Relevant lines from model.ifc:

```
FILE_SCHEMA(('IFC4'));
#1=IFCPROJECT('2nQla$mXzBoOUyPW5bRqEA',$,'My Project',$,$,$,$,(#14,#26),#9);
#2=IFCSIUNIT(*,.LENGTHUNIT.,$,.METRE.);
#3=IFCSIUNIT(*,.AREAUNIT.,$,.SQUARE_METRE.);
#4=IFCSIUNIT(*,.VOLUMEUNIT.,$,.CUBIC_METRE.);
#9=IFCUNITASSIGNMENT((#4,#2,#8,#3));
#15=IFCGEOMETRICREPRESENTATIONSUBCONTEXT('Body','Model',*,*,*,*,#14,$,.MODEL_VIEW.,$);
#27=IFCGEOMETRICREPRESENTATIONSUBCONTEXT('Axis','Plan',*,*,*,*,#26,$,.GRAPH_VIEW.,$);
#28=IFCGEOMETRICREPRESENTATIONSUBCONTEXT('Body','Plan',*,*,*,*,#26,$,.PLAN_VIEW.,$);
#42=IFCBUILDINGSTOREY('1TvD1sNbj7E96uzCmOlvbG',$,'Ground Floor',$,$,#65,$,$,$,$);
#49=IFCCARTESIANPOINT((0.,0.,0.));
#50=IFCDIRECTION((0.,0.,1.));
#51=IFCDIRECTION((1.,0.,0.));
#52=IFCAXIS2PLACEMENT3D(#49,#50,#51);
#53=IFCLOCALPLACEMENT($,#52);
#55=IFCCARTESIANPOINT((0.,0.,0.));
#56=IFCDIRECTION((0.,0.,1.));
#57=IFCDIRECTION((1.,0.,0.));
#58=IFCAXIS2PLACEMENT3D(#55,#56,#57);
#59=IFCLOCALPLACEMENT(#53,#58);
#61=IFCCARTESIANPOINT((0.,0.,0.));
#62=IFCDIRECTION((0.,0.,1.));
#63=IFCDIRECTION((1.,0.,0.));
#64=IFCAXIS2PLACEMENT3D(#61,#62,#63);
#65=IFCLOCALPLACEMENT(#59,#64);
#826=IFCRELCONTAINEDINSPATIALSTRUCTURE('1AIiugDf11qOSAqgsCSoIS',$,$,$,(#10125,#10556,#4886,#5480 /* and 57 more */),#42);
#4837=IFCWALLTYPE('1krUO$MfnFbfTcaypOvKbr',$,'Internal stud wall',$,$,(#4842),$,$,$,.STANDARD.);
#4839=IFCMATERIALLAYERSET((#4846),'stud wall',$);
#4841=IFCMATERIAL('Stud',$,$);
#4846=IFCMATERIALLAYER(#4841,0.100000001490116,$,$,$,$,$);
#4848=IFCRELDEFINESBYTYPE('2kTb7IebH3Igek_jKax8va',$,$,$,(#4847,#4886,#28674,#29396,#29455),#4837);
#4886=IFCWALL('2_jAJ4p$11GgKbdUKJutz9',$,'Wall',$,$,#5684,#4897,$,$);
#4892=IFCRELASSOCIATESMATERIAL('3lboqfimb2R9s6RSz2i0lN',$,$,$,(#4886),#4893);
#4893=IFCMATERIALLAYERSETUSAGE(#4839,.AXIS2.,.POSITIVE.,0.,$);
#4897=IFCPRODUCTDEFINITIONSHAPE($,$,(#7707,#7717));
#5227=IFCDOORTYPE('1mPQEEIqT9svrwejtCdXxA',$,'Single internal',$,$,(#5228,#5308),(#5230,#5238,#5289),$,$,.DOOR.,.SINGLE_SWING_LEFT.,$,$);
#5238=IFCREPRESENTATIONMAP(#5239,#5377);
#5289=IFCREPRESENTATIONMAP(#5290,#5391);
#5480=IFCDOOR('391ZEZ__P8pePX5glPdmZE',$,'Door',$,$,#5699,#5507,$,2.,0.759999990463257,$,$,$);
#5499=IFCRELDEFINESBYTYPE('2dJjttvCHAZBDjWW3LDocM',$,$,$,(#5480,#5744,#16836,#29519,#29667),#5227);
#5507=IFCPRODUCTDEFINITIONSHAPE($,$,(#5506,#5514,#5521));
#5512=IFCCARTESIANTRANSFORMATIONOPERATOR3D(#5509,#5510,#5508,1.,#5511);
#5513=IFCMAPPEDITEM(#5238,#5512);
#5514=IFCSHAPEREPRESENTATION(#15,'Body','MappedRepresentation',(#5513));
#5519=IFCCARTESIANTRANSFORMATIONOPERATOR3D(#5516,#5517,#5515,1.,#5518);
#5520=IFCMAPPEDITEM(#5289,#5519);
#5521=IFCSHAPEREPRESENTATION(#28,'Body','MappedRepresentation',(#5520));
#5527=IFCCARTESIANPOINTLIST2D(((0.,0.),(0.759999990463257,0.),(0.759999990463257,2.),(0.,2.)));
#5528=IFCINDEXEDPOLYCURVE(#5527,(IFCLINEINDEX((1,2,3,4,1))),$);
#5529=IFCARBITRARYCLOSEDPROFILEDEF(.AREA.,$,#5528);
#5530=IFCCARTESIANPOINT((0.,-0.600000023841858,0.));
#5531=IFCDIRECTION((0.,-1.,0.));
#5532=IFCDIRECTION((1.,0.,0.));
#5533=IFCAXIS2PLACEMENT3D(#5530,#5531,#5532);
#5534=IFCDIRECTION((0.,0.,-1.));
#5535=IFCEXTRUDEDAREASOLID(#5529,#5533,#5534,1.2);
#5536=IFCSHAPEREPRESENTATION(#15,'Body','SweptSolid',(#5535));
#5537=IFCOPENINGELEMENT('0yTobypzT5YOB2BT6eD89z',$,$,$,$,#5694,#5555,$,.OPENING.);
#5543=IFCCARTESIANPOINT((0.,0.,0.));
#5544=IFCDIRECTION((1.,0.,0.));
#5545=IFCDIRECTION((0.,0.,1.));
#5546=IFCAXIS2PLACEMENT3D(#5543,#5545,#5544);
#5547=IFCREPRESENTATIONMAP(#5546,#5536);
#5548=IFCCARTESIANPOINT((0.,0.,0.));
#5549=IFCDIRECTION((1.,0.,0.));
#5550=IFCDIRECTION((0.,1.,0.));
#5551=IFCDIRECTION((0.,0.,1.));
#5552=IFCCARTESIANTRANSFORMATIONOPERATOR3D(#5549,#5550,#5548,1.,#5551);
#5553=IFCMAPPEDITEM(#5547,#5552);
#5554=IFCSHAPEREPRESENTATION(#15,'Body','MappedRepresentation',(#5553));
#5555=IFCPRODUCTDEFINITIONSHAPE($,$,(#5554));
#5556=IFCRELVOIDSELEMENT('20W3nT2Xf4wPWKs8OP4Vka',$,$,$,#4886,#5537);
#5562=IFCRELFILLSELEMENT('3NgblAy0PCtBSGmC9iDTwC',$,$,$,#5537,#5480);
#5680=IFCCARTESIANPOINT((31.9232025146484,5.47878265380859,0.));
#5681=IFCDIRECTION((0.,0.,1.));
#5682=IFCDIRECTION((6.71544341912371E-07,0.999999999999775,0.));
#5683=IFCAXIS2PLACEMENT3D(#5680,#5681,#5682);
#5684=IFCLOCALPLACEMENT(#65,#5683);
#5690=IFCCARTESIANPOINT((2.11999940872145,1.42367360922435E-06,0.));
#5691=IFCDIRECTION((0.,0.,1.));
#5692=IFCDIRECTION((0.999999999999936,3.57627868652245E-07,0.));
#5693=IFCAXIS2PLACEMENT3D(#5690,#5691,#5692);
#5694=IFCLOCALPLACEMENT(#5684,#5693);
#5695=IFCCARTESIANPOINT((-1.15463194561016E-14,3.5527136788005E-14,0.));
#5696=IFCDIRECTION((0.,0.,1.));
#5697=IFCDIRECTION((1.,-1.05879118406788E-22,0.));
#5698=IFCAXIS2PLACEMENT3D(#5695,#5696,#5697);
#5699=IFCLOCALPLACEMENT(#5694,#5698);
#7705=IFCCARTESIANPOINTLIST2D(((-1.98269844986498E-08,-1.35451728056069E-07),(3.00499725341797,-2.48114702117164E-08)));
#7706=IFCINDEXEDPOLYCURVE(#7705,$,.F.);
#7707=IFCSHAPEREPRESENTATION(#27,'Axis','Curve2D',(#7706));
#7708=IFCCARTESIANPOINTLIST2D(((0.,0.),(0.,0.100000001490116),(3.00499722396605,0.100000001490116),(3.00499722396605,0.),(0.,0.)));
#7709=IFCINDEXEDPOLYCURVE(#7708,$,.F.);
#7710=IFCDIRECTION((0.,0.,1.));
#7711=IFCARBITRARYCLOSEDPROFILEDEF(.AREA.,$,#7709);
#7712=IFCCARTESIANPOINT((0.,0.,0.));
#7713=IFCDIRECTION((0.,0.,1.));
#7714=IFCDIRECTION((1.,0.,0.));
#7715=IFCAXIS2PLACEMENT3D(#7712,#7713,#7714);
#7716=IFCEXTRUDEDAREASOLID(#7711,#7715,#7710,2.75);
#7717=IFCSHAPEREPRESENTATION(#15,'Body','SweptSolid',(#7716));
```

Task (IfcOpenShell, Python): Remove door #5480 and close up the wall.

```python
import ifcopenshell
import ifcopenshell.api.feature
import ifcopenshell.api.root
import ifcopenshell.geom
import ifcopenshell.util.shape

model = ifcopenshell.open("model.ifc")
settings = ifcopenshell.geom.settings()


def volume(element):
    """Net volume in cubic metres, openings subtracted."""
    shape = ifcopenshell.geom.create_shape(settings, element)
    return ifcopenshell.util.shape.get_volume(shape.geometry)


door = model.by_guid("391ZEZ__P8pePX5glPdmZE")
opening = door.FillsVoids[0].RelatingOpeningElement
wall = opening.VoidsElements[0].RelatingBuildingElement
before = volume(wall)

ifcopenshell.api.root.remove_product(model, product=door)
ifcopenshell.api.feature.remove_feature(model, feature=opening)

after = volume(wall)

print(f"wall volume {before:.3f} -> {after:.3f} m3")

model.write("model_rev.ifc")
```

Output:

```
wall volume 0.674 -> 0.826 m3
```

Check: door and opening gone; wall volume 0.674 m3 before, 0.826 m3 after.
